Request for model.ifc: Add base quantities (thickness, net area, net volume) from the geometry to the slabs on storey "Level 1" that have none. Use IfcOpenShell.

First a look at what the model holds.

```python
import ifcopenshell
import ifcopenshell.util.element
import ifcopenshell.util.unit

model = ifcopenshell.open("model.ifc")
print(model.schema)
for unit_type in ("LENGTHUNIT", "AREAUNIT", "VOLUMEUNIT"):
    print(unit_type, ifcopenshell.util.unit.calculate_unit_scale(model, unit_type))
storey = next(s for s in model.by_type("IfcBuildingStorey") if s.Name == "Level 1")
slabs = [e for e in ifcopenshell.util.element.get_decomposition(storey) if e.is_a("IfcSlab")]
for e in sorted(slabs, key=lambda e: e.id()):
    print(e.id(), e.is_a(), e.Name, list(ifcopenshell.util.element.get_psets(e, qtos_only=True)), sep=" | ")
```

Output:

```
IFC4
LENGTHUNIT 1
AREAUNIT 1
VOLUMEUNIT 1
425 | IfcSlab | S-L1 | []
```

```python
import ifcopenshell
import ifcopenshell.api.pset
import ifcopenshell.geom
import ifcopenshell.util.element
import ifcopenshell.util.shape
import ifcopenshell.util.unit

model = ifcopenshell.open("model.ifc")
unit_scale = ifcopenshell.util.unit.calculate_unit_scale(model)
area_scale = ifcopenshell.util.unit.calculate_unit_scale(model, "AREAUNIT")
volume_scale = ifcopenshell.util.unit.calculate_unit_scale(model, "VOLUMEUNIT")
settings = ifcopenshell.geom.settings()

storey = next(s for s in model.by_type("IfcBuildingStorey") if s.Name == "Level 1")
slabs = [e for e in ifcopenshell.util.element.get_decomposition(storey) if e.is_a("IfcSlab")]

for e in sorted(slabs, key=lambda e: e.id()):
    if ifcopenshell.util.element.get_psets(e, qtos_only=True, should_inherit=False):
        continue
    # Geometry comes back in metres, in the element's own axes.
    shape = ifcopenshell.geom.create_shape(settings, e)
    values = {
        "Width": ifcopenshell.util.shape.get_z(shape.geometry) / unit_scale,
        "NetArea": ifcopenshell.util.shape.get_footprint_area(shape.geometry) / area_scale,
        "NetVolume": ifcopenshell.util.shape.get_volume(shape.geometry) / volume_scale,
    }
    qto = ifcopenshell.api.pset.add_qto(model, product=e, name="Qto_SlabBaseQuantities")
    ifcopenshell.api.pset.edit_qto(model, qto=qto, properties=values)
    print(e.id(), {k: round(v, 3) for k, v in values.items()})

model.write("model_updated.ifc")
```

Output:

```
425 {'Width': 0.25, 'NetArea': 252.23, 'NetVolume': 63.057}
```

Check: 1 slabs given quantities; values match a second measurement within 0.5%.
